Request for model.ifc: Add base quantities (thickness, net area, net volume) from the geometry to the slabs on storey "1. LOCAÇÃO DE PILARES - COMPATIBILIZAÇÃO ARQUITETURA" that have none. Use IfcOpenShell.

First a look at what the model holds.

```python
import ifcopenshell
import ifcopenshell.util.element
import ifcopenshell.util.unit

model = ifcopenshell.open("model.ifc")
print(model.schema)
for unit_type in ("LENGTHUNIT", "AREAUNIT", "VOLUMEUNIT"):
    print(unit_type, ifcopenshell.util.unit.calculate_unit_scale(model, unit_type))
storey = next(s for s in model.by_type("IfcBuildingStorey") if s.Name == "1. LOCAÇÃO DE PILARES - COMPATIBILIZAÇÃO ARQUITETURA")
slabs = [e for e in ifcopenshell.util.element.get_decomposition(storey) if e.is_a("IfcSlab")]
for e in sorted(slabs, key=lambda e: e.id()):
    print(e.id(), e.is_a(), e.Name, list(ifcopenshell.util.element.get_psets(e, qtos_only=True)), sep=" | ")
```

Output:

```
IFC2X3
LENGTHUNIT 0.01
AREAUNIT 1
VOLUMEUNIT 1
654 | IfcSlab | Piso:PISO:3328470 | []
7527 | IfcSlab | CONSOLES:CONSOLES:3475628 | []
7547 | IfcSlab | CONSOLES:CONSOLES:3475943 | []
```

```python
import ifcopenshell
import ifcopenshell.api.pset
import ifcopenshell.geom
import ifcopenshell.util.element
import ifcopenshell.util.shape
import ifcopenshell.util.unit

model = ifcopenshell.open("model.ifc")
unit_scale = ifcopenshell.util.unit.calculate_unit_scale(model)
area_scale = ifcopenshell.util.unit.calculate_unit_scale(model, "AREAUNIT")
volume_scale = ifcopenshell.util.unit.calculate_unit_scale(model, "VOLUMEUNIT")
settings = ifcopenshell.geom.settings()

storey = next(s for s in model.by_type("IfcBuildingStorey") if s.Name == "1. LOCAÇÃO DE PILARES - COMPATIBILIZAÇÃO ARQUITETURA")
slabs = [e for e in ifcopenshell.util.element.get_decomposition(storey) if e.is_a("IfcSlab")]

for e in sorted(slabs, key=lambda e: e.id()):
    if ifcopenshell.util.element.get_psets(e, qtos_only=True, should_inherit=False):
        continue
    # Geometry comes back in metres, in the element's own axes.
    shape = ifcopenshell.geom.create_shape(settings, e)
    values = {
        "Width": ifcopenshell.util.shape.get_z(shape.geometry) / unit_scale,
        "NetArea": ifcopenshell.util.shape.get_footprint_area(shape.geometry) / area_scale,
        "NetVolume": ifcopenshell.util.shape.get_volume(shape.geometry) / volume_scale,
    }
    qto = ifcopenshell.api.pset.add_qto(model, product=e, name="BaseQuantities")
    ifcopenshell.api.pset.edit_qto(model, qto=qto, properties=values)
    print(e.id(), {k: round(v, 3) for k, v in values.items()})

model.write("model_updated.ifc")
```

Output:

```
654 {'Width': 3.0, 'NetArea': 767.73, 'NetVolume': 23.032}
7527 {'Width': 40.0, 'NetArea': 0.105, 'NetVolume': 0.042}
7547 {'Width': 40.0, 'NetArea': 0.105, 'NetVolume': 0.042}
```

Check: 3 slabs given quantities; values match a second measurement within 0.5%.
